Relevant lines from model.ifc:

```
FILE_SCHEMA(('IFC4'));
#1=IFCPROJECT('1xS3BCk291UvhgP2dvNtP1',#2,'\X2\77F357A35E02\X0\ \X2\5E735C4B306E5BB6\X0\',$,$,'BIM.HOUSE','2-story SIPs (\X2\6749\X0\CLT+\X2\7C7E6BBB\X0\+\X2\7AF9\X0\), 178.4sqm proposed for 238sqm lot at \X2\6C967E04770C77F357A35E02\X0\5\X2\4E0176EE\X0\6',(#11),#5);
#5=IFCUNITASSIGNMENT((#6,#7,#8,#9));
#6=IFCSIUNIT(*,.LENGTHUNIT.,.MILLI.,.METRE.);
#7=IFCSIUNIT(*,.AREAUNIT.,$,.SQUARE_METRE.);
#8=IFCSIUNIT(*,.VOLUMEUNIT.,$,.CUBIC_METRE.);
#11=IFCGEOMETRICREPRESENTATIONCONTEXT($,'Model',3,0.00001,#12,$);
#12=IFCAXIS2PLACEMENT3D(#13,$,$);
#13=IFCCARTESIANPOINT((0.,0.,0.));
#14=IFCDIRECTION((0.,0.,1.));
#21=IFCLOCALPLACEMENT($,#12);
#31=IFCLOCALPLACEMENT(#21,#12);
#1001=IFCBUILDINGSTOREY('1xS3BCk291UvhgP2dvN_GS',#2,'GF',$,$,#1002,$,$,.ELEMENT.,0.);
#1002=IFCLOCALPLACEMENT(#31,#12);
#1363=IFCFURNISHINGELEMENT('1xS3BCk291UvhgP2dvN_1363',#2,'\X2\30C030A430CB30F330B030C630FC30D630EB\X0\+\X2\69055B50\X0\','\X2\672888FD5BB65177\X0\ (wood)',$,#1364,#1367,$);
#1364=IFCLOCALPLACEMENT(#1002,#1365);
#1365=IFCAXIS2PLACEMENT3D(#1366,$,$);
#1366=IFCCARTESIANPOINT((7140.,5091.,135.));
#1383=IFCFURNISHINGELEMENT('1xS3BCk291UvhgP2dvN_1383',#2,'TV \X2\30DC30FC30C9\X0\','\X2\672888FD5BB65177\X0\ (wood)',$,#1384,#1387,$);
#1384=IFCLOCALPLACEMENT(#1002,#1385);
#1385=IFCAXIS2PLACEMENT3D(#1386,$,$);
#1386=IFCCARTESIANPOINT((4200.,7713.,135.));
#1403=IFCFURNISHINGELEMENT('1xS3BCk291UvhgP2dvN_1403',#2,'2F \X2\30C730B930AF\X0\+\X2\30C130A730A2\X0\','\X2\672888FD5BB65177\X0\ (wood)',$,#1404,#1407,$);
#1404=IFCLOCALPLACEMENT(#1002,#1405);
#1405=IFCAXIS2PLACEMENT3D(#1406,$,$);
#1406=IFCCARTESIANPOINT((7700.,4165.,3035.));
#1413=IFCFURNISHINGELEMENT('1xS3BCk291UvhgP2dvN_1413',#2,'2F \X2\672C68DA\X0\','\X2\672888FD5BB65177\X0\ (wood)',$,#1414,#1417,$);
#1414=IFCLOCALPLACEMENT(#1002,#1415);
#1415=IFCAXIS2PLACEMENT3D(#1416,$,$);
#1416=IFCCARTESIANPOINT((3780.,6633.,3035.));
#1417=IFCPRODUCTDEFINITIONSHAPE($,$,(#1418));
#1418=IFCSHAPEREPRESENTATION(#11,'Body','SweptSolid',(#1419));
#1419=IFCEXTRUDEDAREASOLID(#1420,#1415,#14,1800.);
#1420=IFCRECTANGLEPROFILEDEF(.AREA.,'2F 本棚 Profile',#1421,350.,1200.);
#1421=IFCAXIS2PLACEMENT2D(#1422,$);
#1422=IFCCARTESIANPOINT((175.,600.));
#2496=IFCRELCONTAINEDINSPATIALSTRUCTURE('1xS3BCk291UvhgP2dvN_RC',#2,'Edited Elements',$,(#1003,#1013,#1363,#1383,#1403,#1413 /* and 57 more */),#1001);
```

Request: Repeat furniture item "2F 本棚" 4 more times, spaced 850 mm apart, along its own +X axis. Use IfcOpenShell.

```python
import ifcopenshell
import ifcopenshell.api.geometry
import ifcopenshell.api.root
import ifcopenshell.util.element
import ifcopenshell.util.placement
import ifcopenshell.util.unit

model = ifcopenshell.open("model.ifc")
unit_scale = ifcopenshell.util.unit.calculate_unit_scale(model)


def reuse_history(source, copy):
    """copy_class also copies each property set's owner history, people and application; keep the originals."""
    for rel in copy.IsDefinedBy:
        if rel.is_a("IfcRelDefinesByProperties") and (history := rel.RelatingPropertyDefinition.OwnerHistory):
            rel.RelatingPropertyDefinition.OwnerHistory = source.OwnerHistory
            ifcopenshell.util.element.remove_deep2(model, history)


source = model.by_id(1413)
base = ifcopenshell.util.placement.get_local_placement(source.ObjectPlacement)
step = base[:3, 0] * 0.85 / unit_scale

for i in range(1, 5):
    copy = ifcopenshell.api.root.copy_class(model, product=source)
    copy.Representation = ifcopenshell.util.element.copy_deep(
        model, source.Representation, exclude=["IfcGeometricRepresentationContext", "IfcRepresentationMap"]
    )
    reuse_history(source, copy)
    matrix = base.copy()
    matrix[:3, 3] += i * step
    print("added at", matrix[:3, 3].round(3) + 0.0)
    ifcopenshell.api.geometry.edit_object_placement(model, product=copy, matrix=matrix, is_si=False)

model.write("model_v2.ifc")
```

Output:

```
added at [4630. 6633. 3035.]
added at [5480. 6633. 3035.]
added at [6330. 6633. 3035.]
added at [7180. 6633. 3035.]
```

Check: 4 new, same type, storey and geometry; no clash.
